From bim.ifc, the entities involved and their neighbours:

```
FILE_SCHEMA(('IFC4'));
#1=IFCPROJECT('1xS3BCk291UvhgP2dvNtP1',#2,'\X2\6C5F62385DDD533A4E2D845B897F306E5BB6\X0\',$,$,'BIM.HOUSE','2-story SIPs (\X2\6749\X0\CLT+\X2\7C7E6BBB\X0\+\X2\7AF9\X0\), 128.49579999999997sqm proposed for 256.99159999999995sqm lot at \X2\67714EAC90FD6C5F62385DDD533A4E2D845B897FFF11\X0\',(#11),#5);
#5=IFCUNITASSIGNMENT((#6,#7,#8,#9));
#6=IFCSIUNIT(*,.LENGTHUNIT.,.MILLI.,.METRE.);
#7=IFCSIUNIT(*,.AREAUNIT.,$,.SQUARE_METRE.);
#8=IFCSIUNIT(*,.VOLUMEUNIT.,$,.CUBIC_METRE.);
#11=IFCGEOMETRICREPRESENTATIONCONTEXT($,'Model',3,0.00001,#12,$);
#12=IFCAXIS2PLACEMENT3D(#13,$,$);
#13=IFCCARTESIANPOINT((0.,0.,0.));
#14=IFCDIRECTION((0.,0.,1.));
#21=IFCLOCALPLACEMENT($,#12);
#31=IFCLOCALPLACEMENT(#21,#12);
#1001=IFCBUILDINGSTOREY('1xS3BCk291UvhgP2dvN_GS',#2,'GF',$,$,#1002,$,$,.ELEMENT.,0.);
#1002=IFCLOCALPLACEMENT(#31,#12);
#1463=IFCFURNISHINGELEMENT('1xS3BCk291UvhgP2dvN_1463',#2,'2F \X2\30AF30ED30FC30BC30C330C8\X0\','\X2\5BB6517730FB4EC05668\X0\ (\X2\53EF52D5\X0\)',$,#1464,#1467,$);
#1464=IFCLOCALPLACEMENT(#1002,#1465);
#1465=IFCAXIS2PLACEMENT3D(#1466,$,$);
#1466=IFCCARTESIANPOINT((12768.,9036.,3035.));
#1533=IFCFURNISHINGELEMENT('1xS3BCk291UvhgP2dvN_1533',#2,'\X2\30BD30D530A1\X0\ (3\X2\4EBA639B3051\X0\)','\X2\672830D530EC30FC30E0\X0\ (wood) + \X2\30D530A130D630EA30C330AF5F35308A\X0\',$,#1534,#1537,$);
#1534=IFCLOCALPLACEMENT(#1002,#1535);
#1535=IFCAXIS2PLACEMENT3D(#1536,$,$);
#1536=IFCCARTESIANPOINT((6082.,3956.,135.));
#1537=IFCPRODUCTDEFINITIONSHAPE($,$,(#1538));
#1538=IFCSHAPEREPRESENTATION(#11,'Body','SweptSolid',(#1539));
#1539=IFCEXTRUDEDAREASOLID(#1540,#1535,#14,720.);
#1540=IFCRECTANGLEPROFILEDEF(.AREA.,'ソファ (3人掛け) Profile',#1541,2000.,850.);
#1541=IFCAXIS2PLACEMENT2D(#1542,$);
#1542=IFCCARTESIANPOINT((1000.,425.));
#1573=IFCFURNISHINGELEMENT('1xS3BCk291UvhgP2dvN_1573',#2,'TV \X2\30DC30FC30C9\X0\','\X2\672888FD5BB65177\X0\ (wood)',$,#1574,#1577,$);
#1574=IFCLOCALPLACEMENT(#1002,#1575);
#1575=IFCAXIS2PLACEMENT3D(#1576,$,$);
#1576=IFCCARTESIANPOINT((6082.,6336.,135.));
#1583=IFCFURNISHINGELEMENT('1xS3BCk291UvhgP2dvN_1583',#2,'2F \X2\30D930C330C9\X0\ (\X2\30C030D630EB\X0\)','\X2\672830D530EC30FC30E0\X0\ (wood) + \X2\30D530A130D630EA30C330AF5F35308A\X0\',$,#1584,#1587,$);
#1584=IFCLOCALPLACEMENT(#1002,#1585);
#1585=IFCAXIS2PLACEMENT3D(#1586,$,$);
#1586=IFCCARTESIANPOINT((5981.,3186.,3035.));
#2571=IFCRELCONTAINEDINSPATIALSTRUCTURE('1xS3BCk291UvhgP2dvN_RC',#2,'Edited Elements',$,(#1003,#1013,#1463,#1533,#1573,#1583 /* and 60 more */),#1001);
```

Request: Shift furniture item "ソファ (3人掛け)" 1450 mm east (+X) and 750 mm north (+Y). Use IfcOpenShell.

```python
import ifcopenshell
import ifcopenshell.api.geometry
import ifcopenshell.util.placement

model = ifcopenshell.open("bim.ifc")

item = model.by_guid("1xS3BCk291UvhgP2dvN_1533")
matrix = ifcopenshell.util.placement.get_local_placement(item.ObjectPlacement)
matrix[0, 3] += 1450.0
matrix[1, 3] += 750.0
ifcopenshell.api.geometry.edit_object_placement(model, product=item, matrix=matrix, is_si=False)

print(ifcopenshell.util.placement.get_local_placement(item.ObjectPlacement).round(3) + 0.0)

model.write("bim_edited.ifc")
```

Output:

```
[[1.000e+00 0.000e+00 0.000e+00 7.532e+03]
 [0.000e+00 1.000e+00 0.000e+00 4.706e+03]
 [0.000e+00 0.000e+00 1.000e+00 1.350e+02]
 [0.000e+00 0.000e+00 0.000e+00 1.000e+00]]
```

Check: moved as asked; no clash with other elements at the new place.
